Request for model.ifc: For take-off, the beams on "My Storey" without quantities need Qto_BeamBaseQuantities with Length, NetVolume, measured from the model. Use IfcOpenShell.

First a look at what the model holds.

```python
import ifcopenshell
import ifcopenshell.util.element
import ifcopenshell.util.unit

model = ifcopenshell.open("model.ifc")
print(model.schema)
for unit_type in ("LENGTHUNIT", "AREAUNIT", "VOLUMEUNIT"):
    print(unit_type, ifcopenshell.util.unit.calculate_unit_scale(model, unit_type))
storey = next(s for s in model.by_type("IfcBuildingStorey") if s.Name == "My Storey")
beams = [e for e in ifcopenshell.util.element.get_decomposition(storey) if e.is_a("IfcBeam")]
for e in sorted(beams, key=lambda e: e.id()):
    print(e.id(), e.is_a(), e.Name, list(ifcopenshell.util.element.get_psets(e, qtos_only=True)), sep=" | ")
```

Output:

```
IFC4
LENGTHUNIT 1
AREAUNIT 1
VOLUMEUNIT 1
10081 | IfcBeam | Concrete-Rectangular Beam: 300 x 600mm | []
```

```python
import ifcopenshell
import ifcopenshell.api.pset
import ifcopenshell.geom
import ifcopenshell.util.element
import ifcopenshell.util.shape
import ifcopenshell.util.unit

model = ifcopenshell.open("model.ifc")
unit_scale = ifcopenshell.util.unit.calculate_unit_scale(model)
volume_scale = ifcopenshell.util.unit.calculate_unit_scale(model, "VOLUMEUNIT")
settings = ifcopenshell.geom.settings()

storey = next(s for s in model.by_type("IfcBuildingStorey") if s.Name == "My Storey")
beams = [e for e in ifcopenshell.util.element.get_decomposition(storey) if e.is_a("IfcBeam")]

for e in sorted(beams, key=lambda e: e.id()):
    if ifcopenshell.util.element.get_psets(e, qtos_only=True, should_inherit=False):
        continue
    # Geometry comes back in metres, in the element's own axes.
    shape = ifcopenshell.geom.create_shape(settings, e)
    values = {
        "Length": ifcopenshell.util.shape.get_max_xyz(shape.geometry) / unit_scale,
        "NetVolume": ifcopenshell.util.shape.get_volume(shape.geometry) / volume_scale,
    }
    qto = ifcopenshell.api.pset.add_qto(model, product=e, name="Qto_BeamBaseQuantities")
    ifcopenshell.api.pset.edit_qto(model, qto=qto, properties=values)
    print(e.id(), {k: round(v, 3) for k, v in values.items()})

model.write("model_edited.ifc")
```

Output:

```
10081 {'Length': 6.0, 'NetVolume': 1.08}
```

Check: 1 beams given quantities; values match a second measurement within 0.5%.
